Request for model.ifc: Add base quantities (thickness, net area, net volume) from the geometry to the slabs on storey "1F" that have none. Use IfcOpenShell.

First a look at what the model holds.

```python
import ifcopenshell
import ifcopenshell.util.element
import ifcopenshell.util.unit

model = ifcopenshell.open("model.ifc")
print(model.schema)
for unit_type in ("LENGTHUNIT", "AREAUNIT", "VOLUMEUNIT"):
    print(unit_type, ifcopenshell.util.unit.calculate_unit_scale(model, unit_type))
storey = next(s for s in model.by_type("IfcBuildingStorey") if s.Name == "1F")
slabs = [e for e in ifcopenshell.util.element.get_decomposition(storey) if e.is_a("IfcSlab")]
for e in sorted(slabs, key=lambda e: e.id()):
    print(e.id(), e.is_a(), e.Name, list(ifcopenshell.util.element.get_psets(e, qtos_only=True)), sep=" | ")
```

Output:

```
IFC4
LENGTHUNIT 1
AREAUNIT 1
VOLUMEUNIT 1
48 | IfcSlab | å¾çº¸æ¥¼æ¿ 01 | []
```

```python
import ifcopenshell
import ifcopenshell.api.pset
import ifcopenshell.geom
import ifcopenshell.util.element
import ifcopenshell.util.shape
import ifcopenshell.util.unit

model = ifcopenshell.open("model.ifc")
unit_scale = ifcopenshell.util.unit.calculate_unit_scale(model)
area_scale = ifcopenshell.util.unit.calculate_unit_scale(model, "AREAUNIT")
volume_scale = ifcopenshell.util.unit.calculate_unit_scale(model, "VOLUMEUNIT")
settings = ifcopenshell.geom.settings()

storey = next(s for s in model.by_type("IfcBuildingStorey") if s.Name == "1F")
slabs = [e for e in ifcopenshell.util.element.get_decomposition(storey) if e.is_a("IfcSlab")]

for e in sorted(slabs, key=lambda e: e.id()):
    if ifcopenshell.util.element.get_psets(e, qtos_only=True, should_inherit=False):
        continue
    # Geometry comes back in metres, in the element's own axes.
    shape = ifcopenshell.geom.create_shape(settings, e)
    values = {
        "Width": ifcopenshell.util.shape.get_z(shape.geometry) / unit_scale,
        "NetArea": ifcopenshell.util.shape.get_footprint_area(shape.geometry) / area_scale,
        "NetVolume": ifcopenshell.util.shape.get_volume(shape.geometry) / volume_scale,
    }
    qto = ifcopenshell.api.pset.add_qto(model, product=e, name="Qto_SlabBaseQuantities")
    ifcopenshell.api.pset.edit_qto(model, qto=qto, properties=values)
    print(e.id(), {k: round(v, 3) for k, v in values.items()})

model.write("model_rev.ifc")
```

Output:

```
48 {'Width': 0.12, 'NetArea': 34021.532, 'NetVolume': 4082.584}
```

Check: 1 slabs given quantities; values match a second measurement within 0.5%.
